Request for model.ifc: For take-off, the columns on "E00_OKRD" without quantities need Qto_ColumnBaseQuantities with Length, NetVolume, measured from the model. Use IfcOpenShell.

First a look at what the model holds.

```python
import ifcopenshell
import ifcopenshell.util.element
import ifcopenshell.util.unit

model = ifcopenshell.open("model.ifc")
print(model.schema)
for unit_type in ("LENGTHUNIT", "AREAUNIT", "VOLUMEUNIT"):
    print(unit_type, ifcopenshell.util.unit.calculate_unit_scale(model, unit_type))
storey = next(s for s in model.by_type("IfcBuildingStorey") if s.Name == "E00_OKRD")
columns = [e for e in ifcopenshell.util.element.get_decomposition(storey) if e.is_a("IfcColumn")]
for e in sorted(columns, key=lambda e: e.id()):
    print(e.id(), e.is_a(), e.Name, list(ifcopenshell.util.element.get_psets(e, qtos_only=True)), sep=" | ")
```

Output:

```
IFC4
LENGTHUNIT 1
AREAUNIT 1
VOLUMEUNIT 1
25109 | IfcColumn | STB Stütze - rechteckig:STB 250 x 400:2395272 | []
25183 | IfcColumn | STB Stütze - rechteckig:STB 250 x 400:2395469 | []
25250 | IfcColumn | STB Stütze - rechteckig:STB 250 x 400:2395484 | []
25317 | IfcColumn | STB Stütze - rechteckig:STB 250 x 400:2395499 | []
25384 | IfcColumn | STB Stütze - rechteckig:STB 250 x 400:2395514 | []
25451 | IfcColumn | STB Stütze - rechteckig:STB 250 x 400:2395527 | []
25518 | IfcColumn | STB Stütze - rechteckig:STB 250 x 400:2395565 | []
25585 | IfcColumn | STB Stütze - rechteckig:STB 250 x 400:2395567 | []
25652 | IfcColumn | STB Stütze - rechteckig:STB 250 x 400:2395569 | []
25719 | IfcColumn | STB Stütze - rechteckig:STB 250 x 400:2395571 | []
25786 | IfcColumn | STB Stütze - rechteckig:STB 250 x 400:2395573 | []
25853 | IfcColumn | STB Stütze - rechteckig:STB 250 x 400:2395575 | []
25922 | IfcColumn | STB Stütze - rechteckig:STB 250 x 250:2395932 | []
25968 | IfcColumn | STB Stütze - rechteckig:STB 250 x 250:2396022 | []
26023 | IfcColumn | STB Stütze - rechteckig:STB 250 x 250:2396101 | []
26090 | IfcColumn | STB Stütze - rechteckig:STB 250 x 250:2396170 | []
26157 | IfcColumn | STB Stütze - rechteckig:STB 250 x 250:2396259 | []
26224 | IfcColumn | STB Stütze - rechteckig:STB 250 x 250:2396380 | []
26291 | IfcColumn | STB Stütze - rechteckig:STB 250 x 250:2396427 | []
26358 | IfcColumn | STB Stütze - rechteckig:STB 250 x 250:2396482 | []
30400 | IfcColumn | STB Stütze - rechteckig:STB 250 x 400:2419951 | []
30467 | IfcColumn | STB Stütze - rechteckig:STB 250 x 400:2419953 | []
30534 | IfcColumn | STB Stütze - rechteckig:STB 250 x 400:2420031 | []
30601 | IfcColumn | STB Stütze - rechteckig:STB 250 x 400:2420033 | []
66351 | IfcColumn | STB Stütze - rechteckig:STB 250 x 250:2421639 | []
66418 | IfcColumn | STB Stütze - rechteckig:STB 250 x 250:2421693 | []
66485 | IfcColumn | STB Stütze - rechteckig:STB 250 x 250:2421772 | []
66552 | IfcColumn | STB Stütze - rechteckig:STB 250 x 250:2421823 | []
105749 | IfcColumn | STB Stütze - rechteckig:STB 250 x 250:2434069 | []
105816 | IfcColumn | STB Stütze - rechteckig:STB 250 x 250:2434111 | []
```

```python
import ifcopenshell
import ifcopenshell.api.pset
import ifcopenshell.geom
import ifcopenshell.util.element
import ifcopenshell.util.shape
import ifcopenshell.util.unit

model = ifcopenshell.open("model.ifc")
unit_scale = ifcopenshell.util.unit.calculate_unit_scale(model)
volume_scale = ifcopenshell.util.unit.calculate_unit_scale(model, "VOLUMEUNIT")
settings = ifcopenshell.geom.settings()

storey = next(s for s in model.by_type("IfcBuildingStorey") if s.Name == "E00_OKRD")
columns = [e for e in ifcopenshell.util.element.get_decomposition(storey) if e.is_a("IfcColumn")]

for e in sorted(columns, key=lambda e: e.id()):
    if ifcopenshell.util.element.get_psets(e, qtos_only=True, should_inherit=False):
        continue
    # Geometry comes back in metres, in the element's own axes.
    shape = ifcopenshell.geom.create_shape(settings, e)
    values = {
        "Length": ifcopenshell.util.shape.get_z(shape.geometry) / unit_scale,
        "NetVolume": ifcopenshell.util.shape.get_volume(shape.geometry) / volume_scale,
    }
    qto = ifcopenshell.api.pset.add_qto(model, product=e, name="Qto_ColumnBaseQuantities")
    ifcopenshell.api.pset.edit_qto(model, qto=qto, properties=values)
    print(e.id(), {k: round(v, 3) for k, v in values.items()})

model.write("model_v2.ifc")
```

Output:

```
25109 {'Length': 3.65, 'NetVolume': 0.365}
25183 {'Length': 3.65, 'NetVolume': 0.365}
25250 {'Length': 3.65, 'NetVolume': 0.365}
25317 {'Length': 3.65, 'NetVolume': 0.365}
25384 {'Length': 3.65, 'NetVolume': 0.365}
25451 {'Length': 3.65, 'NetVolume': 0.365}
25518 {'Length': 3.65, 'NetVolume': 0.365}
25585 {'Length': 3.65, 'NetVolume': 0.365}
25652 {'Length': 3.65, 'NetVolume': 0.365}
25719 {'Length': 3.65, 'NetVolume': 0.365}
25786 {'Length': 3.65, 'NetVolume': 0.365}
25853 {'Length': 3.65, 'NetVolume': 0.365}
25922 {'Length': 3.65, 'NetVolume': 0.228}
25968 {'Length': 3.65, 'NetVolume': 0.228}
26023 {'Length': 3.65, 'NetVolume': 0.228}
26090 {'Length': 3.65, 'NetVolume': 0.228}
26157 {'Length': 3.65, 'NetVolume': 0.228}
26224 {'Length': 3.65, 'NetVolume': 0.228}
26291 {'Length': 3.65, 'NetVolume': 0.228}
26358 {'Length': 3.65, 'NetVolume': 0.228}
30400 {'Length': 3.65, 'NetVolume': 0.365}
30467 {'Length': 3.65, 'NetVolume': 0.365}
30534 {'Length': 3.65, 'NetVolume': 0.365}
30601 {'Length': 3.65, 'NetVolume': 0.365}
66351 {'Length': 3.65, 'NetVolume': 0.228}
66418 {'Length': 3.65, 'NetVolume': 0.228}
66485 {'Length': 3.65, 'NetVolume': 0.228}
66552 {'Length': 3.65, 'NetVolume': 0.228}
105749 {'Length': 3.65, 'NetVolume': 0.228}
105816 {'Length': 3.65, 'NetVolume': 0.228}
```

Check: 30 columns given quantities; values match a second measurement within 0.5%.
